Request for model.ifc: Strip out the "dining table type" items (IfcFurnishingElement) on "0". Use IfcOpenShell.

First a look at what the model holds.

```python
import ifcopenshell
import ifcopenshell.util.element

model = ifcopenshell.open("model.ifc")
print(model.schema)
storey = next(s for s in model.by_type("IfcBuildingStorey") if s.Name == "0")
furniture = [e for e in ifcopenshell.util.element.get_decomposition(storey) if e.is_a("IfcFurnishingElement")]
seen = {}
for e in furniture:
    element_type = ifcopenshell.util.element.get_type(e)
    name = element_type.Name if element_type not in (None, e) else None
    seen[name] = seen.get(name, 0) + 1
for name, count in sorted(seen.items(), key=str):
    print(count, "x", name)
```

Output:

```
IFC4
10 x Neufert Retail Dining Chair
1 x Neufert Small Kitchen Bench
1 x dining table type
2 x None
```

```python
import ifcopenshell
import ifcopenshell.api.root
import ifcopenshell.util.element

model = ifcopenshell.open("model.ifc")

storey = next(s for s in model.by_type("IfcBuildingStorey") if s.Name == "0")
furniture = [e for e in ifcopenshell.util.element.get_decomposition(storey) if e.is_a("IfcFurnishingElement")]
targets = [e for e in furniture if (t := ifcopenshell.util.element.get_type(e)) not in (None, e) and t.Name == "dining table type"]

for e in targets:
    ifcopenshell.api.root.remove_product(model, product=e)
print(len(targets), "removed")

model.write("model_updated.ifc")
```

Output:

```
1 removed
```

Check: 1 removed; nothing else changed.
